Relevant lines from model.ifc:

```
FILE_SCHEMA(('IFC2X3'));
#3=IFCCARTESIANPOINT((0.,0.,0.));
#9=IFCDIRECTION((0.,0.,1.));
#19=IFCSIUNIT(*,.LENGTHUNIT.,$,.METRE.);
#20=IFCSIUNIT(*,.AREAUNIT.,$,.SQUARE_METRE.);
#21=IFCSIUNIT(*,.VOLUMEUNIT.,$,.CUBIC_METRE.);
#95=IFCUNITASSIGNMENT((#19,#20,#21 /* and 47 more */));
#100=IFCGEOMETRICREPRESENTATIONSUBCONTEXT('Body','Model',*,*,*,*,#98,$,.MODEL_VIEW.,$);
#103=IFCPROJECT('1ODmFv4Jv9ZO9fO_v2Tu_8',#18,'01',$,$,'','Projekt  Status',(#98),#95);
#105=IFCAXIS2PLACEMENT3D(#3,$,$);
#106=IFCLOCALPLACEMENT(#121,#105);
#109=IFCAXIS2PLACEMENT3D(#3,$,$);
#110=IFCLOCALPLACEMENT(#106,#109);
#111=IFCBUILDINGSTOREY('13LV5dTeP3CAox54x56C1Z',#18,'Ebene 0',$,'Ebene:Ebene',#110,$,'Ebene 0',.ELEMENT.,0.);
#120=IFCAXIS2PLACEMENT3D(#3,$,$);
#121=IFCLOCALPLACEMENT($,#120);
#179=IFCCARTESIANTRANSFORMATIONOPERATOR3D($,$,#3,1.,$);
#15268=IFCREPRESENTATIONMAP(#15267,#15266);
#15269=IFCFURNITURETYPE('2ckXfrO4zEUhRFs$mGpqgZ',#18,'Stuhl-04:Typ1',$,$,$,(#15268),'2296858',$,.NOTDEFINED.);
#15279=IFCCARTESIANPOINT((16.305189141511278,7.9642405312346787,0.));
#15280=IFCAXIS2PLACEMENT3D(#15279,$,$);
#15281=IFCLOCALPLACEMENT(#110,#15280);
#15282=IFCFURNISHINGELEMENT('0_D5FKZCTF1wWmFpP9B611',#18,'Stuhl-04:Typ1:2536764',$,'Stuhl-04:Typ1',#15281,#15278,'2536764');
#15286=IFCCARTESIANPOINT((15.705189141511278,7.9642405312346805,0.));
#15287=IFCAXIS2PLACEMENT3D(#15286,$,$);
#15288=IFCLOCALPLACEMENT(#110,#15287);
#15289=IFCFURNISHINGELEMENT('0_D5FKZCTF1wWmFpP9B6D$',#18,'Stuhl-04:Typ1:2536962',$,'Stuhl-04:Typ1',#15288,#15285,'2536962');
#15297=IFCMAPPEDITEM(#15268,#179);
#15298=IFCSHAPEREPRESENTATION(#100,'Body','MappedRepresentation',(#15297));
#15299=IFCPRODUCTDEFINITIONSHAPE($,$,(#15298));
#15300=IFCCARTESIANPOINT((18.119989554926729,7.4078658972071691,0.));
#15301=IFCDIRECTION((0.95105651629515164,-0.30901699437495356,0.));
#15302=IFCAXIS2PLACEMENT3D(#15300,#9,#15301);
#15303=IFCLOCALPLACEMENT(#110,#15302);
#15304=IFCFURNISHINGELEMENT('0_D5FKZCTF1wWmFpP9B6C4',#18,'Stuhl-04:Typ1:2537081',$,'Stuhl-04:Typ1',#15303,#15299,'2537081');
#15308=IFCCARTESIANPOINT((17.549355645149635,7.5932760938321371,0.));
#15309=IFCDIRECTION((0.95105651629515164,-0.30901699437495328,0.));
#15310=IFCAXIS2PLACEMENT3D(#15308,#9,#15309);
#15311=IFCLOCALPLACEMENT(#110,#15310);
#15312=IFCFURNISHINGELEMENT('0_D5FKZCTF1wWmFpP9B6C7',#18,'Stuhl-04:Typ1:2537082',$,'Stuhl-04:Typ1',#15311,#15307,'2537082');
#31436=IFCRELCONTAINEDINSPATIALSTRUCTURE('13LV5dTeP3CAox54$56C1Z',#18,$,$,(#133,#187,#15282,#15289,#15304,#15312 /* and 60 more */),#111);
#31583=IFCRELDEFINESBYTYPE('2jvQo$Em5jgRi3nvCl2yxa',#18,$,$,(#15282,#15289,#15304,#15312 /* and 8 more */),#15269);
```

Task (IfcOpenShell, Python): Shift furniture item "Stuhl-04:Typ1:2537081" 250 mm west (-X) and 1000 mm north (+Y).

```python
import ifcopenshell
import ifcopenshell.api.geometry
import ifcopenshell.util.placement
import ifcopenshell.util.unit

model = ifcopenshell.open("model.ifc")
unit_scale = ifcopenshell.util.unit.calculate_unit_scale(model)

item = model.by_guid("0_D5FKZCTF1wWmFpP9B6C4")
matrix = ifcopenshell.util.placement.get_local_placement(item.ObjectPlacement)
matrix[0, 3] -= 0.25 / unit_scale
matrix[1, 3] += 1 / unit_scale
ifcopenshell.api.geometry.edit_object_placement(model, product=item, matrix=matrix, is_si=False)

print(ifcopenshell.util.placement.get_local_placement(item.ObjectPlacement).round(3) + 0.0)

model.write("model_edited.ifc")
```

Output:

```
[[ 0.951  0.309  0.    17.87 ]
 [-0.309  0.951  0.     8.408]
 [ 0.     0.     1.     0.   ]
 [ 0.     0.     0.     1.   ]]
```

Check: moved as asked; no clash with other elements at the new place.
